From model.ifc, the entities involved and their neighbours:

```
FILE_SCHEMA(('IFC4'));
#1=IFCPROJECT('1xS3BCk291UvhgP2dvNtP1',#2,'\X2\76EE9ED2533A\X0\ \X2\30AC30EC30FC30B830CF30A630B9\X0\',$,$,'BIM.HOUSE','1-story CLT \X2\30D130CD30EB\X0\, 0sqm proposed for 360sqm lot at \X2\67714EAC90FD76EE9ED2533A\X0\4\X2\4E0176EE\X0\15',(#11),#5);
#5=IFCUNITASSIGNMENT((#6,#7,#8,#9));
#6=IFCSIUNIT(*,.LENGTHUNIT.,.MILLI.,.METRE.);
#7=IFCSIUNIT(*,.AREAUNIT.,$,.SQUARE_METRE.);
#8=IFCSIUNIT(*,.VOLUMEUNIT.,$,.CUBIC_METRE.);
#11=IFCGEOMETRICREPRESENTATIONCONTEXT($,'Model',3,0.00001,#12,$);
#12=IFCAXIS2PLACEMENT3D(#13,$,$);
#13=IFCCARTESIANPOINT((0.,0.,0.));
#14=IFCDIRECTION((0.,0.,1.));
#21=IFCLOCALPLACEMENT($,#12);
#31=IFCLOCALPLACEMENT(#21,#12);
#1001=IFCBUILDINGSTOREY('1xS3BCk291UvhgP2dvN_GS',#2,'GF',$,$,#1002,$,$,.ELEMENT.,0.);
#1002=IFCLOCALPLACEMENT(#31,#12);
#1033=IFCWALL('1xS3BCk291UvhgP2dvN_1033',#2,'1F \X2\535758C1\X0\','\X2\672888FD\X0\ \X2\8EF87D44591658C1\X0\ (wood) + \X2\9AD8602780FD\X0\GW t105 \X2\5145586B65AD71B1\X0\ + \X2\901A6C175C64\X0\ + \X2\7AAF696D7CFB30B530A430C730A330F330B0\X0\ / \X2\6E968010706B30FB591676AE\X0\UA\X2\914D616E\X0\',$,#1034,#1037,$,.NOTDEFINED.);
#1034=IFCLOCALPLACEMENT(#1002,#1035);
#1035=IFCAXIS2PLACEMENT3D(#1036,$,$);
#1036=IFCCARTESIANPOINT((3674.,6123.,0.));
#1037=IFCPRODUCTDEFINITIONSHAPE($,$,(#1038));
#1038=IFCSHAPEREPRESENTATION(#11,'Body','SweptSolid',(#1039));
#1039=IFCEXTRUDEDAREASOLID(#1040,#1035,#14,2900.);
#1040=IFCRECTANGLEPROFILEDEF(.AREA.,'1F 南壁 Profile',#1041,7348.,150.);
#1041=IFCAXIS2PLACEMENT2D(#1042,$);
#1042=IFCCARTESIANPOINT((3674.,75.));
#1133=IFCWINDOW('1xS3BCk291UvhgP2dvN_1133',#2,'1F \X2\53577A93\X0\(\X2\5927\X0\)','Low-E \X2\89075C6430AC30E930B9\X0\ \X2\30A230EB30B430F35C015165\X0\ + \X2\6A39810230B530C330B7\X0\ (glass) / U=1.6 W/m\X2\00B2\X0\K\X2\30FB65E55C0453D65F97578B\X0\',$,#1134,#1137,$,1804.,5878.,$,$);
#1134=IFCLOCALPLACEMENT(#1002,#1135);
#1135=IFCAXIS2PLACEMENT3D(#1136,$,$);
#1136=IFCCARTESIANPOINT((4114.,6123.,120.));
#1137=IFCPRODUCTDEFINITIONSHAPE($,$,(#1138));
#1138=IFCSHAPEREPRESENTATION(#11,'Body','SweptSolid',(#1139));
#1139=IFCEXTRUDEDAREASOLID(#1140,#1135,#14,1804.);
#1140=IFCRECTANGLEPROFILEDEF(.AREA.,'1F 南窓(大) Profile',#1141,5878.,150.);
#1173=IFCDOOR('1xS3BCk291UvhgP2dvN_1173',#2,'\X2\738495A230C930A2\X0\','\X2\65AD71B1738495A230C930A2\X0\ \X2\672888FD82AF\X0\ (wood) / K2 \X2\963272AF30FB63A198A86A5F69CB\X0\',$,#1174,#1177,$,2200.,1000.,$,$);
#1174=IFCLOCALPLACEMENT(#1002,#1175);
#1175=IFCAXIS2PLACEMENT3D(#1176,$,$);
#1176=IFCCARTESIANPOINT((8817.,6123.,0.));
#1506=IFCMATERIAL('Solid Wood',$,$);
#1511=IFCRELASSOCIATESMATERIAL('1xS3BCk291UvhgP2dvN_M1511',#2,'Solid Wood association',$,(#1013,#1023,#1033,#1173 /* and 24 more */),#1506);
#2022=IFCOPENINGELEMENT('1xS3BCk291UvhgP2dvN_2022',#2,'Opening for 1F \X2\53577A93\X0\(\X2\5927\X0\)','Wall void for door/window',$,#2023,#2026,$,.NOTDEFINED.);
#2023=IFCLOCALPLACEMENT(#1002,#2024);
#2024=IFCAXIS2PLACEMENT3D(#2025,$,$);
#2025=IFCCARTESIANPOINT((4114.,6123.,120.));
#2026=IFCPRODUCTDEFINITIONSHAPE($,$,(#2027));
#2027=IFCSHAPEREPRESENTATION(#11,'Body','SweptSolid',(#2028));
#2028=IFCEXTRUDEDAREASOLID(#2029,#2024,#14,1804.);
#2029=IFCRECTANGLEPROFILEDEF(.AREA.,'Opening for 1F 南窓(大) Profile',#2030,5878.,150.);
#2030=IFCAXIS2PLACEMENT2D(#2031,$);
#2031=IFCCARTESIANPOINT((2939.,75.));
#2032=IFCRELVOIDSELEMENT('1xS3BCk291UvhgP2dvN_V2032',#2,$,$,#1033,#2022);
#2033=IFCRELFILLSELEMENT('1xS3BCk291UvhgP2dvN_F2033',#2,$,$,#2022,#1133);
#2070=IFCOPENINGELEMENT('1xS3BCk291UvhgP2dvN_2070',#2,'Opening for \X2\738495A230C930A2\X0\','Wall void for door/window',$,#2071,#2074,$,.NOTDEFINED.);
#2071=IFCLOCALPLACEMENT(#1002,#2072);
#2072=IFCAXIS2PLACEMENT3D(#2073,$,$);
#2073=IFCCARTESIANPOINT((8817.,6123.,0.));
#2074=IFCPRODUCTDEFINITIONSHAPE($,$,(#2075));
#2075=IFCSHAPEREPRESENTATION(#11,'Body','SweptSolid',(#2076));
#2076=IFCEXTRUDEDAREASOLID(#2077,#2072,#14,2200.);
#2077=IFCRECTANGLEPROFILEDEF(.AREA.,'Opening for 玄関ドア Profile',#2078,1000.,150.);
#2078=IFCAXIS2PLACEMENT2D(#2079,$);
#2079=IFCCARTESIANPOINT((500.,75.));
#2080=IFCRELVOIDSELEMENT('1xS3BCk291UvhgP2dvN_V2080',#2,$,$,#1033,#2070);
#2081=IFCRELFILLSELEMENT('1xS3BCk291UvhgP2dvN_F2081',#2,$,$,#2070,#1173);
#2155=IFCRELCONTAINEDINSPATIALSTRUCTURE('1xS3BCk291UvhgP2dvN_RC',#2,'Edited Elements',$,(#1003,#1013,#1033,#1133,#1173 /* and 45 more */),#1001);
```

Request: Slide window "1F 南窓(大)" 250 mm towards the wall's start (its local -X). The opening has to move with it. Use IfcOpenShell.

```python
import ifcopenshell
import ifcopenshell.api.geometry
import ifcopenshell.util.placement

model = ifcopenshell.open("model.ifc")

window = model.by_guid("1xS3BCk291UvhgP2dvN_1133")
opening = window.FillsVoids[0].RelatingOpeningElement
wall = opening.VoidsElements[0].RelatingBuildingElement

wall_matrix = ifcopenshell.util.placement.get_local_placement(wall.ObjectPlacement)
shift = wall_matrix[:3, 0] * -250.0
before = ifcopenshell.util.placement.get_local_placement(window.ObjectPlacement)[:3, 3].copy()

# The window is not placed relative to its opening, so move both.
for product in (opening, window):
    matrix = ifcopenshell.util.placement.get_local_placement(product.ObjectPlacement)
    matrix[:3, 3] += shift
    ifcopenshell.api.geometry.edit_object_placement(model, product=product, matrix=matrix, is_si=False)

after = ifcopenshell.util.placement.get_local_placement(window.ObjectPlacement)[:3, 3]
print("window moved by", (after - before).round(3) + 0.0)

model.write("model_v2.ifc")
```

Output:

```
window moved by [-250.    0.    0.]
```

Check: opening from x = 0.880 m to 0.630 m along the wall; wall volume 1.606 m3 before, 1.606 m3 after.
